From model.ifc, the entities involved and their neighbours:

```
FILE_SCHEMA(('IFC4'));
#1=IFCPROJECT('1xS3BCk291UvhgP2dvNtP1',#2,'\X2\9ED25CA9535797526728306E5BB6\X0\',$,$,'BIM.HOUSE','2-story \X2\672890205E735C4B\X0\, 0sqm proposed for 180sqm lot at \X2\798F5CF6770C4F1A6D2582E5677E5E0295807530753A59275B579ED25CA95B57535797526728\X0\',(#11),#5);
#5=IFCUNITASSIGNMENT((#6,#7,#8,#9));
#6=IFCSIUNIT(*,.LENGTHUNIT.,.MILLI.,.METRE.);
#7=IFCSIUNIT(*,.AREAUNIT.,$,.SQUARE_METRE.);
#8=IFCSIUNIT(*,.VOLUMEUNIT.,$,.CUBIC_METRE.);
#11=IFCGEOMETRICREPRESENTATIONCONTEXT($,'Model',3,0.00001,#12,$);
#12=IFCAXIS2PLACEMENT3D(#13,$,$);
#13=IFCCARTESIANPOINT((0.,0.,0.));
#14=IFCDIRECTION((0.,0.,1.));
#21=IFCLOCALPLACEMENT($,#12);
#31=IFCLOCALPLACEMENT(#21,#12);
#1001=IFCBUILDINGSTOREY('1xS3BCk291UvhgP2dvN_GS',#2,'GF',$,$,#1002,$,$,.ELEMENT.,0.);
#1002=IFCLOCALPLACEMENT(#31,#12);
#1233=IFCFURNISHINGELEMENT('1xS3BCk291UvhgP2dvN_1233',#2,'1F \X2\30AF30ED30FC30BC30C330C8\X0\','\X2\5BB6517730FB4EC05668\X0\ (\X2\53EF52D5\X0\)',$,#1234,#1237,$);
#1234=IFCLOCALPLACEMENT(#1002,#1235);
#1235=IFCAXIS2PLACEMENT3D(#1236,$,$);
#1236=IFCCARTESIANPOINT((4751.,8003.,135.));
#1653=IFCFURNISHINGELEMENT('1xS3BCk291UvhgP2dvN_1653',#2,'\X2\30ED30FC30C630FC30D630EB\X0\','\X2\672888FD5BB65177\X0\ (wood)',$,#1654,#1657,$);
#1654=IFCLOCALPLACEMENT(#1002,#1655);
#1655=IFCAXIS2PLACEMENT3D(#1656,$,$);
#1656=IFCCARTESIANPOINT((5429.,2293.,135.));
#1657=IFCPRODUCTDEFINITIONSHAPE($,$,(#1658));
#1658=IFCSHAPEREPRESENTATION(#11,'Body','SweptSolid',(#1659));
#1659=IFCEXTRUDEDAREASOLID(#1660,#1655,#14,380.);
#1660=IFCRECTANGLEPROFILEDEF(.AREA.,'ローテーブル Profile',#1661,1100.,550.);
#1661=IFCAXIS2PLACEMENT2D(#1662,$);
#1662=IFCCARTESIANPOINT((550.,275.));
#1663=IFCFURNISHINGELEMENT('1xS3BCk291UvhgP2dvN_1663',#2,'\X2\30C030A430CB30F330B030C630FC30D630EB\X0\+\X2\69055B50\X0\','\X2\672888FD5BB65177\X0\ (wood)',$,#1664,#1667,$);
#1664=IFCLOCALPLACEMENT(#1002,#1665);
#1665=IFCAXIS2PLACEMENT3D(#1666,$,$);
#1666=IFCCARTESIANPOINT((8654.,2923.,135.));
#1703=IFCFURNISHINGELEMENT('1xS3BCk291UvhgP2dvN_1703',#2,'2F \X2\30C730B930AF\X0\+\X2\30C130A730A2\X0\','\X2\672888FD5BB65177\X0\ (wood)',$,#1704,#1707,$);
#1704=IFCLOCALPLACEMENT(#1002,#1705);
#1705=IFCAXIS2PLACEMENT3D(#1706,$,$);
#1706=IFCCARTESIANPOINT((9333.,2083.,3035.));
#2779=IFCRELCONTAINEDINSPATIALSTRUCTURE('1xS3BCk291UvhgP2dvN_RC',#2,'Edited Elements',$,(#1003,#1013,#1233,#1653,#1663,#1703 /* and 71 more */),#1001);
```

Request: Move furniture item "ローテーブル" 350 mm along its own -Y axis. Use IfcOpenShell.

```python
import ifcopenshell
import ifcopenshell.api.geometry
import ifcopenshell.util.placement
import ifcopenshell.util.unit

model = ifcopenshell.open("model.ifc")
unit_scale = ifcopenshell.util.unit.calculate_unit_scale(model)

item = model.by_id(1653)
matrix = ifcopenshell.util.placement.get_local_placement(item.ObjectPlacement)
matrix[:3, 3] -= matrix[:3, 1] * 0.35 / unit_scale
ifcopenshell.api.geometry.edit_object_placement(model, product=item, matrix=matrix, is_si=False)

print(ifcopenshell.util.placement.get_local_placement(item.ObjectPlacement).round(3) + 0.0)

model.write("model_updated.ifc")
```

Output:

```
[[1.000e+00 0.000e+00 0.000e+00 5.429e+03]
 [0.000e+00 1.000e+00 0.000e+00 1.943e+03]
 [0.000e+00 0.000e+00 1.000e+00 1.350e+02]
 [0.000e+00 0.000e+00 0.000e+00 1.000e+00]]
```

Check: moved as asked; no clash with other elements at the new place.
